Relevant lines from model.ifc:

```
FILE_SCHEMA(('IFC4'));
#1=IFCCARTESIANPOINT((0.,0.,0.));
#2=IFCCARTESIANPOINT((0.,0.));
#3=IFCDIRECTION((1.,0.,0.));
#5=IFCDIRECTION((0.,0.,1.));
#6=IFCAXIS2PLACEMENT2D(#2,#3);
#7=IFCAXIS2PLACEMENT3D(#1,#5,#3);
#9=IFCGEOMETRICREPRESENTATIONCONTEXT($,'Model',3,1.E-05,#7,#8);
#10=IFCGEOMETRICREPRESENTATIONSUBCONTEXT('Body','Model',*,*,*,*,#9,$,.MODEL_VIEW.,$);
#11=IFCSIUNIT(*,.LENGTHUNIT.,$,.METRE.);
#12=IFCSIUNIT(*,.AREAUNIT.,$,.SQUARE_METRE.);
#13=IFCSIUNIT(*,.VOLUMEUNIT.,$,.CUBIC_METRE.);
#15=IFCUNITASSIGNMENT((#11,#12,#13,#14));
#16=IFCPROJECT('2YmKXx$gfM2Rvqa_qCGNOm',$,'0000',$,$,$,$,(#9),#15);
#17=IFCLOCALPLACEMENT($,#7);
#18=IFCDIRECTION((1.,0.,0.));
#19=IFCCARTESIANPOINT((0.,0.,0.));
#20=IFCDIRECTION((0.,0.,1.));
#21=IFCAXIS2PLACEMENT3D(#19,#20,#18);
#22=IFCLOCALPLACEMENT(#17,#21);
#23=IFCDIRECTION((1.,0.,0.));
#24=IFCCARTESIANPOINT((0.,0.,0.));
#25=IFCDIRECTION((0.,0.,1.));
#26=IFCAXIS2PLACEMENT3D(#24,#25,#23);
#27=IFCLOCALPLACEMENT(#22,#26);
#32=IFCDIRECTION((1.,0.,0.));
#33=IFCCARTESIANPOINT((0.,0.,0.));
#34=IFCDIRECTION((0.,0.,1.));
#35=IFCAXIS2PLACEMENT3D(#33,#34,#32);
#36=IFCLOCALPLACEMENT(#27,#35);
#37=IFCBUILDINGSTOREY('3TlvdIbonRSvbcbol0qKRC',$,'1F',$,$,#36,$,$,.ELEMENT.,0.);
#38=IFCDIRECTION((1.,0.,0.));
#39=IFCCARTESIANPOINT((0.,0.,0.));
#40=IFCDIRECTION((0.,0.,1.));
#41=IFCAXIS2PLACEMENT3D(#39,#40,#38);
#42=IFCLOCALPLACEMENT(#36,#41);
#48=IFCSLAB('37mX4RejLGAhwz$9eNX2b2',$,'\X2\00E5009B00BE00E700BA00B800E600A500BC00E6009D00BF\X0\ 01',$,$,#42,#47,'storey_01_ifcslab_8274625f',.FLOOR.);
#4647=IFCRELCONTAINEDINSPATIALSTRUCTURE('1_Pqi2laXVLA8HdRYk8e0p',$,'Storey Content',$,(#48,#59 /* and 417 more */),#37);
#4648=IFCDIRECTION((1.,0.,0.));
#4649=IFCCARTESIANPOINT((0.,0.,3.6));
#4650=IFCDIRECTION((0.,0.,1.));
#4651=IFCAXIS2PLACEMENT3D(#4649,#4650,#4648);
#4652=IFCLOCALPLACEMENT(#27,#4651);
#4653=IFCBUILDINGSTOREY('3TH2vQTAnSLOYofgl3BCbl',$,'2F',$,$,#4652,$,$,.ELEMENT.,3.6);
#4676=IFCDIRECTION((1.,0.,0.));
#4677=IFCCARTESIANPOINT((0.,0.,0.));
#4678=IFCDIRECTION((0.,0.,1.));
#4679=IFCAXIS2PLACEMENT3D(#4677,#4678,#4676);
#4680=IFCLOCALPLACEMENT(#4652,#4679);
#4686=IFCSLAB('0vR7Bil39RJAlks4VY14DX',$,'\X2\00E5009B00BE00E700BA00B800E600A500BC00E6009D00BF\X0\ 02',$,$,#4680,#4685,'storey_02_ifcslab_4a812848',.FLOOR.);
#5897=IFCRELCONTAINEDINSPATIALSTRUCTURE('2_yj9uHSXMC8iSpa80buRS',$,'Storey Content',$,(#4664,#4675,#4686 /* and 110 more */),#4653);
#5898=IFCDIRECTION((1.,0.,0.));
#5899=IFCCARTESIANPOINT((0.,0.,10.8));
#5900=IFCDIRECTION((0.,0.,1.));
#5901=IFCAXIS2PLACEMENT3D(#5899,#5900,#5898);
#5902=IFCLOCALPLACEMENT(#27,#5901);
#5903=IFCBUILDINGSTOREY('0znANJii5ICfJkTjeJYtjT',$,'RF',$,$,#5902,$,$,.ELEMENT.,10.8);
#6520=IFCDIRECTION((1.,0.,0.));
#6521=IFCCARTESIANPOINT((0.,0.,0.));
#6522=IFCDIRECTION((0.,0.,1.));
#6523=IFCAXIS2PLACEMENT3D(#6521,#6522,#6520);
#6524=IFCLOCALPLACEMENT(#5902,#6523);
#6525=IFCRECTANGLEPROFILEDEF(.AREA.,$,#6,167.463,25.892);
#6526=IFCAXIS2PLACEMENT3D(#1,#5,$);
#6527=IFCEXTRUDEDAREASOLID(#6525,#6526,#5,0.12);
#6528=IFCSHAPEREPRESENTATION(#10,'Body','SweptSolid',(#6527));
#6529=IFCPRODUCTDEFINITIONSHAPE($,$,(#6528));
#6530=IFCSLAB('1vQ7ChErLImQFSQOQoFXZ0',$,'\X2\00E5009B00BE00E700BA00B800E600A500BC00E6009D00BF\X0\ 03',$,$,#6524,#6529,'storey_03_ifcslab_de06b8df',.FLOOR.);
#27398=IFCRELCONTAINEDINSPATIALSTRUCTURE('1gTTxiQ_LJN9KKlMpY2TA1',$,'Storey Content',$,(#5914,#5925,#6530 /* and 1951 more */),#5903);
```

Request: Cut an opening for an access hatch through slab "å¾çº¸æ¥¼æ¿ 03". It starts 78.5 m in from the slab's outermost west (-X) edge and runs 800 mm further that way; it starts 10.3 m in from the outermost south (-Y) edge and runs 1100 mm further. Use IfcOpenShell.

```python
import numpy as np
import ifcopenshell
import ifcopenshell.api.feature
import ifcopenshell.api.geometry
import ifcopenshell.api.root
import ifcopenshell.geom
import ifcopenshell.util.placement
import ifcopenshell.util.representation
import ifcopenshell.util.shape
import ifcopenshell.util.unit

model = ifcopenshell.open("model.ifc")
unit_scale = ifcopenshell.util.unit.calculate_unit_scale(model)
settings = ifcopenshell.geom.settings()


def volume(element):
    """Net volume in cubic metres, openings subtracted."""
    shape = ifcopenshell.geom.create_shape(settings, element)
    return ifcopenshell.util.shape.get_volume(shape.geometry)


slab = model.by_guid("1vQ7ChErLImQFSQOQoFXZ0")
before = volume(slab)

# Extent in the slab's own axes, in metres. The edges named are its -X and -Y sides.
slab_shape = ifcopenshell.geom.create_shape(settings, slab)
vertices = ifcopenshell.util.shape.get_vertices(slab_shape.geometry)
x_min, y_min, bottom = vertices.min(axis=0)
top = vertices[:, 2].max()

opening = ifcopenshell.api.root.create_entity(model, ifc_class="IfcOpeningElement", name="Access hatch opening", predefined_type="OPENING")
context = ifcopenshell.util.representation.get_context(model, "Model", "Body", "MODEL_VIEW")
width, depth = 0.8, 1.1
outline = [(0.0, 0.0), (width, 0.0), (width, depth), (0.0, depth), (0.0, 0.0)]
# Overshoot both faces by 50 mm so the cut is clean.
shape = ifcopenshell.api.geometry.add_slab_representation(
    model, context=context, depth=top - bottom + 0.1, polyline=outline
)
ifcopenshell.api.geometry.assign_representation(model, product=opening, representation=shape)

matrix = ifcopenshell.util.placement.get_local_placement(slab.ObjectPlacement)
matrix[:, 3] = matrix @ np.append(np.array([x_min + 78.5, y_min + 10.3, bottom - 0.05]) / unit_scale, 1.0)
ifcopenshell.api.geometry.edit_object_placement(model, product=opening, matrix=matrix, is_si=False)
ifcopenshell.api.feature.add_feature(model, feature=opening, element=slab)

after = volume(slab)

print(f"slab volume {before:.3f} -> {after:.3f} m3")

model.write("model_rev.ifc")
```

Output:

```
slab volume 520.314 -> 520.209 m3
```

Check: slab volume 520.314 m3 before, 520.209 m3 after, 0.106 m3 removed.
